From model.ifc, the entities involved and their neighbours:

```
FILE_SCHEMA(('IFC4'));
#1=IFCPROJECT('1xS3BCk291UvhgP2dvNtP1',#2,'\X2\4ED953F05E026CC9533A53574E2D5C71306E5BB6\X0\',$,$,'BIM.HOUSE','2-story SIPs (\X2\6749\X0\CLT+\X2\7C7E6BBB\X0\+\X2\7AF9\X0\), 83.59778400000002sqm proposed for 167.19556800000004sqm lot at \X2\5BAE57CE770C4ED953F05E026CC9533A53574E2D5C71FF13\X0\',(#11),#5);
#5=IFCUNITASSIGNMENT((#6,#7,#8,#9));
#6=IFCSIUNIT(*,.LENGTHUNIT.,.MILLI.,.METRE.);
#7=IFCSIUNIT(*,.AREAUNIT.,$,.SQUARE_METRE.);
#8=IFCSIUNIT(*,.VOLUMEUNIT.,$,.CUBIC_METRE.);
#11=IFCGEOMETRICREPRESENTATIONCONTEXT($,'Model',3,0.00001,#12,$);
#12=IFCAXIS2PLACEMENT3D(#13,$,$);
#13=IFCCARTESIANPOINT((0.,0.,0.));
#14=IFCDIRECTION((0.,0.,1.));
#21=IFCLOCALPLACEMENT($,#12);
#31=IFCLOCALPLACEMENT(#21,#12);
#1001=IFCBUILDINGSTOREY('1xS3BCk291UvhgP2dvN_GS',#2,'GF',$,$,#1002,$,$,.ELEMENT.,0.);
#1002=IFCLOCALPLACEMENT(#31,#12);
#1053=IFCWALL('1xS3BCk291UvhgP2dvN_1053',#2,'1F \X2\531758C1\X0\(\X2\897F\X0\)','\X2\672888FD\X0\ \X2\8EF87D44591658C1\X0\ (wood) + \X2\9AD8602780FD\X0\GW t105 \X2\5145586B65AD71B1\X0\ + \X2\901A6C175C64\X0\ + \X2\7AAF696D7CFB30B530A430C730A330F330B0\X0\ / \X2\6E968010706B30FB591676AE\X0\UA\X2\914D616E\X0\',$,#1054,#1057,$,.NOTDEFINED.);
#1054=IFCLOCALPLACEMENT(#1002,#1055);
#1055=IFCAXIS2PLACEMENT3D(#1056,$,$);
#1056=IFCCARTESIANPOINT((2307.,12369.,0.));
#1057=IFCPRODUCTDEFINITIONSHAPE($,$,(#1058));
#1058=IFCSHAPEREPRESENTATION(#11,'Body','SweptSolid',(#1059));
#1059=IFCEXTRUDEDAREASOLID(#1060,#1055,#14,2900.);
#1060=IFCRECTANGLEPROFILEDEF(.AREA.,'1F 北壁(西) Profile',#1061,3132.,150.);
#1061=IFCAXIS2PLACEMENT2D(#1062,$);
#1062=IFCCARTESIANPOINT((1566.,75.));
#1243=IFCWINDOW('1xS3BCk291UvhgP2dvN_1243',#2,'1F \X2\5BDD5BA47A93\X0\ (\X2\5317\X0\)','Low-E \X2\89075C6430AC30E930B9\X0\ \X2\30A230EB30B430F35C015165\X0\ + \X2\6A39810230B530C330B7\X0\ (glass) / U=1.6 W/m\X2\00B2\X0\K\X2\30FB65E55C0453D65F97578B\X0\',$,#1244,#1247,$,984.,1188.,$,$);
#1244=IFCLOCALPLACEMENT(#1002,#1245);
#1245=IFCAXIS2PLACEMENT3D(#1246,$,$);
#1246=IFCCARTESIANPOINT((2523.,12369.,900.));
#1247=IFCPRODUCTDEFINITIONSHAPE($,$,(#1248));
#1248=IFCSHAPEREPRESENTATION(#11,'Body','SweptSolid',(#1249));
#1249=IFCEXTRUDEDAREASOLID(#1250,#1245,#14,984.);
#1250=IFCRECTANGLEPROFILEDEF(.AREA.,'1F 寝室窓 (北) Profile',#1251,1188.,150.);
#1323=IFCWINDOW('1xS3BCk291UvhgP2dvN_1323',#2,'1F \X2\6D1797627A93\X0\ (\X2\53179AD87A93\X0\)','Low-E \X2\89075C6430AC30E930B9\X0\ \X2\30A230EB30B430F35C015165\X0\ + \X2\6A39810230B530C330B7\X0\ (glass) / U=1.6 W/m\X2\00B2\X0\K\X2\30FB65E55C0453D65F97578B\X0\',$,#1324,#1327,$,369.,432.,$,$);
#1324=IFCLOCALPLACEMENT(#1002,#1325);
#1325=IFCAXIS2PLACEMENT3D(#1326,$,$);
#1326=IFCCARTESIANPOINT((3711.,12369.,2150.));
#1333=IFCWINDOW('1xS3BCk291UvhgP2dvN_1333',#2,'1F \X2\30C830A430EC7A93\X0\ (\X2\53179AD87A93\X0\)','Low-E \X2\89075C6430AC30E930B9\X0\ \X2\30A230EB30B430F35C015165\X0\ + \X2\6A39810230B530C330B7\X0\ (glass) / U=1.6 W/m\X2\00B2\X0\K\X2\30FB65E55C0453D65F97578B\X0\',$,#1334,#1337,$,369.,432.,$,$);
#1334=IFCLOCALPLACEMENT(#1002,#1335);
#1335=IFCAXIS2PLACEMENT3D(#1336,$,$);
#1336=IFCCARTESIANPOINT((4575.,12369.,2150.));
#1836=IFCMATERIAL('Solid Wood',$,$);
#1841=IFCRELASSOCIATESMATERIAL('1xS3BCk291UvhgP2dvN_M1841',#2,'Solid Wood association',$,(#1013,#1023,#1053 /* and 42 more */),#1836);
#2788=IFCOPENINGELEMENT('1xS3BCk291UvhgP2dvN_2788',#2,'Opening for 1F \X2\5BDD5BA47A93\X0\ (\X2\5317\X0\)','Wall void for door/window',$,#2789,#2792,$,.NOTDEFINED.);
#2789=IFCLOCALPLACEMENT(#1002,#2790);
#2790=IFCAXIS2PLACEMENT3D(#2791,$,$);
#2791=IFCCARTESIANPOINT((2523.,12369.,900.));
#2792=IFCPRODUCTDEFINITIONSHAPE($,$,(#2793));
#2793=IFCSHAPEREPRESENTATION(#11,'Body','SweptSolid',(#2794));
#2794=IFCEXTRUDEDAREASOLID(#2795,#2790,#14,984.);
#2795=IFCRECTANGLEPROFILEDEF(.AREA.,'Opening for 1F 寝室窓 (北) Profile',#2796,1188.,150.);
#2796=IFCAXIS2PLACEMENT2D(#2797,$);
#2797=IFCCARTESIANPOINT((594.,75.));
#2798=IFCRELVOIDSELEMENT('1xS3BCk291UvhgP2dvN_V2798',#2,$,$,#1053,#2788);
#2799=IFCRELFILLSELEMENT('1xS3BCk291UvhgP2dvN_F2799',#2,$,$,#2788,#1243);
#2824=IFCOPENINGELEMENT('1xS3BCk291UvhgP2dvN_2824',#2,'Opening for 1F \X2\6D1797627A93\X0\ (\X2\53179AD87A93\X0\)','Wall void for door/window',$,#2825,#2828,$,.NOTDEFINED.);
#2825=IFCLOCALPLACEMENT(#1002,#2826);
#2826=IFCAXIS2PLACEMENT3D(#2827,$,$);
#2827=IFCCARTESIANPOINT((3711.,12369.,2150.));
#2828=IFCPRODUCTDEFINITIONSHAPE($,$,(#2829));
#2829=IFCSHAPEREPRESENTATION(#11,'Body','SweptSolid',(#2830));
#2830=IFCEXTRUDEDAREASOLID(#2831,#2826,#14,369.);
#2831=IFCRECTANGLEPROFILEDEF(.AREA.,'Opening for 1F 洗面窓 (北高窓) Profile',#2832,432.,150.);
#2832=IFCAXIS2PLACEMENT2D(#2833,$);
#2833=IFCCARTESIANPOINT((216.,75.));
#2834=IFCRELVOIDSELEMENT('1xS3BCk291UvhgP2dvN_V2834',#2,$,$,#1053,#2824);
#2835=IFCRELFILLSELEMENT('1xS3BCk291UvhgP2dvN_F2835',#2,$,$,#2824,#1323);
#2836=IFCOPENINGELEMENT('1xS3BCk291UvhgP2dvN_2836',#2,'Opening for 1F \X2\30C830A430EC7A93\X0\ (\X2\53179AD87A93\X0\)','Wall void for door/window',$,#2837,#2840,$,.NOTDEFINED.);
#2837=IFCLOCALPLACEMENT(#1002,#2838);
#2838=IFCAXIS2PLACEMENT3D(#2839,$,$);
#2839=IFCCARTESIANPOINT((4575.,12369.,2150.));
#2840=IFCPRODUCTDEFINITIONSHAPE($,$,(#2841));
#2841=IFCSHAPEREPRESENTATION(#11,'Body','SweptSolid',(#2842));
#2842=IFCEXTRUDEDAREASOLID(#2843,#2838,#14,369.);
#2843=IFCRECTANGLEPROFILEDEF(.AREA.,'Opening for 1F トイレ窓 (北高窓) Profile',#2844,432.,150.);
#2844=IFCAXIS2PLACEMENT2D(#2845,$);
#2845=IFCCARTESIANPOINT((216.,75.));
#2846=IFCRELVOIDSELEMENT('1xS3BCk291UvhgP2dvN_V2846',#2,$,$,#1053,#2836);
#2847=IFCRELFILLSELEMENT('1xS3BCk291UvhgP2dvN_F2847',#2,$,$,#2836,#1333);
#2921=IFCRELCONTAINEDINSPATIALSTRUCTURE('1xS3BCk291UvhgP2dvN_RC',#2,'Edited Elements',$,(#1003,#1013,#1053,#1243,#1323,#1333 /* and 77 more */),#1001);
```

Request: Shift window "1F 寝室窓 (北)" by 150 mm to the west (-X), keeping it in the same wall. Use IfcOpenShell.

```python
import ifcopenshell
import ifcopenshell.api.geometry
import ifcopenshell.util.placement
import ifcopenshell.util.unit

model = ifcopenshell.open("model.ifc")
unit_scale = ifcopenshell.util.unit.calculate_unit_scale(model)

window = model.by_guid("1xS3BCk291UvhgP2dvN_1243")
opening = window.FillsVoids[0].RelatingOpeningElement
wall = opening.VoidsElements[0].RelatingBuildingElement

wall_matrix = ifcopenshell.util.placement.get_local_placement(wall.ObjectPlacement)
shift = wall_matrix[:3, 0] * -0.15 / unit_scale
before = ifcopenshell.util.placement.get_local_placement(window.ObjectPlacement)[:3, 3].copy()

# The window is not placed relative to its opening, so move both.
for product in (opening, window):
    matrix = ifcopenshell.util.placement.get_local_placement(product.ObjectPlacement)
    matrix[:3, 3] += shift
    ifcopenshell.api.geometry.edit_object_placement(model, product=product, matrix=matrix, is_si=False)

after = ifcopenshell.util.placement.get_local_placement(window.ObjectPlacement)[:3, 3]
print("window moved by", (after - before).round(3) + 0.0)

model.write("model_rev.ifc")
```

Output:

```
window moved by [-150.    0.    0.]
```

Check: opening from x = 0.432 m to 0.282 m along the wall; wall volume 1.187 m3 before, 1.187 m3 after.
